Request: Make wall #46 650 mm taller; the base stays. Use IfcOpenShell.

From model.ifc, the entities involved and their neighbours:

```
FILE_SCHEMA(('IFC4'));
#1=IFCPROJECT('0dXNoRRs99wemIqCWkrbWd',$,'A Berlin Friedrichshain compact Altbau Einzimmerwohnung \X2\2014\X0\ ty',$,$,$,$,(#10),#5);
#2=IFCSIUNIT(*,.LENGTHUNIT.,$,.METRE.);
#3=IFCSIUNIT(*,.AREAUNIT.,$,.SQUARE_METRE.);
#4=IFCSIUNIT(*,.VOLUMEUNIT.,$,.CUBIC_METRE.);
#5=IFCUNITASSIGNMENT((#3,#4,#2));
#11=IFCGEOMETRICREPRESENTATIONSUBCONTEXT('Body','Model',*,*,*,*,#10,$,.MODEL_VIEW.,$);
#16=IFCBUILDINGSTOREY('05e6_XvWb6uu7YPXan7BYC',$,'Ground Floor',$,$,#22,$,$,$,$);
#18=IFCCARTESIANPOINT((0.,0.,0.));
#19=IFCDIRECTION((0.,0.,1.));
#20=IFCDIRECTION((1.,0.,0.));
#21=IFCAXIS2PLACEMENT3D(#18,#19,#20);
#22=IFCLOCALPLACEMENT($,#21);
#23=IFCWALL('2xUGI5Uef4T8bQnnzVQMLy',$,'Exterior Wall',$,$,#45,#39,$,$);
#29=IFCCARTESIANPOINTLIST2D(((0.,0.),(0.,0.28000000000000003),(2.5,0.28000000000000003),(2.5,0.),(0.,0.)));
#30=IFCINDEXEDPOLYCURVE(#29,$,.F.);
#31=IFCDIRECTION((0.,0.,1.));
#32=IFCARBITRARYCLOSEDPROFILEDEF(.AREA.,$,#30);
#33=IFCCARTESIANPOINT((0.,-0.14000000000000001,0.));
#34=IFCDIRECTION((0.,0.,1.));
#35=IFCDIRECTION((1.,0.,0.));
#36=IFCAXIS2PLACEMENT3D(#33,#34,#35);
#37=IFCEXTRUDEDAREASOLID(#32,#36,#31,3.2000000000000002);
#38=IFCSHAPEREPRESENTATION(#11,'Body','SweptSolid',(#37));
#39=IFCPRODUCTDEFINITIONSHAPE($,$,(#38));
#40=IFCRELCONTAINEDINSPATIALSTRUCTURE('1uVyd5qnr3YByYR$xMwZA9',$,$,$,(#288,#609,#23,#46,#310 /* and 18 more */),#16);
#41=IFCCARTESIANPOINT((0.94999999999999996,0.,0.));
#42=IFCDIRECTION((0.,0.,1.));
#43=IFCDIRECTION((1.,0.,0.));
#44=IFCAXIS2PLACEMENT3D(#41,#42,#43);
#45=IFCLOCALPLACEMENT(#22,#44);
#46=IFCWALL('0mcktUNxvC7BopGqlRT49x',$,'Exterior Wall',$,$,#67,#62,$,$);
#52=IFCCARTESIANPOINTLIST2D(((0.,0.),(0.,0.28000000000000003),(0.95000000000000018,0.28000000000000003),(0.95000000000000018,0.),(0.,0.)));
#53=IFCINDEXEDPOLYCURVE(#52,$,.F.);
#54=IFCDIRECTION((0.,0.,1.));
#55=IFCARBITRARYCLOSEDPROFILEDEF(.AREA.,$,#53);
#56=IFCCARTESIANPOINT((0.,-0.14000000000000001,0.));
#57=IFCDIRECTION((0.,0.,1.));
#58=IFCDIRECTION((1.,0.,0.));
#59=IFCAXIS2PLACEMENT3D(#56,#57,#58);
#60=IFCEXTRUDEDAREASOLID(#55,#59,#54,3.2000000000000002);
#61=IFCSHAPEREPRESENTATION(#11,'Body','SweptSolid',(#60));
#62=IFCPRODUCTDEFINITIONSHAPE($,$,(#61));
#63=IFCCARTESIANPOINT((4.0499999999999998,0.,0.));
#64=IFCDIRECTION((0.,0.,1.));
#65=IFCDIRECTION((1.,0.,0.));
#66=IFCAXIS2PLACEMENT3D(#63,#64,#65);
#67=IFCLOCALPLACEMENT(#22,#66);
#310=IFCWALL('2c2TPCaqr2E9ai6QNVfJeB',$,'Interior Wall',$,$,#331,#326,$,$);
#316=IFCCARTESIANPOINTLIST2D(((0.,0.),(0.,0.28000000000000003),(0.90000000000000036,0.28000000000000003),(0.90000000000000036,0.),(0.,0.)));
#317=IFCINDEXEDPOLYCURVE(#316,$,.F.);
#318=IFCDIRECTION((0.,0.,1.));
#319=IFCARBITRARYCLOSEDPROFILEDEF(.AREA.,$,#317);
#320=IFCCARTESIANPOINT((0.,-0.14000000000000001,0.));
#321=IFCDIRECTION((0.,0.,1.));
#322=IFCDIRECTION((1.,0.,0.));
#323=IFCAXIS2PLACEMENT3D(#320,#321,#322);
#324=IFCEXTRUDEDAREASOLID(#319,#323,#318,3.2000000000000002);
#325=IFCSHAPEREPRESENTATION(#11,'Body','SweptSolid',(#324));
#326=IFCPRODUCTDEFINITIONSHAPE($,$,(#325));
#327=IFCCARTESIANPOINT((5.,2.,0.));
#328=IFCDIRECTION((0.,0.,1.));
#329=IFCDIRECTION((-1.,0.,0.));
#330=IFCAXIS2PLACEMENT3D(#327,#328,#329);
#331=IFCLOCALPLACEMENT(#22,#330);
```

```python
import ifcopenshell
import ifcopenshell.geom
import ifcopenshell.util.representation
import ifcopenshell.util.shape
import ifcopenshell.util.unit

model = ifcopenshell.open("model.ifc")
unit_scale = ifcopenshell.util.unit.calculate_unit_scale(model)
settings = ifcopenshell.geom.settings()


def volume(element):
    """Net volume in cubic metres, openings subtracted."""
    shape = ifcopenshell.geom.create_shape(settings, element)
    return ifcopenshell.util.shape.get_volume(shape.geometry)


wall = model.by_guid("0mcktUNxvC7BopGqlRT49x")
before = volume(wall)

body = ifcopenshell.util.representation.get_representation(wall, "Model", "Body")
solid = body.Items[0]
old_height = solid.Depth
solid.Depth += 0.65 / unit_scale
after = volume(wall)

print(f"height {old_height:g} -> {solid.Depth:g}, volume {before:.3f} -> {after:.3f} m3")

model.write("model_updated.ifc")
```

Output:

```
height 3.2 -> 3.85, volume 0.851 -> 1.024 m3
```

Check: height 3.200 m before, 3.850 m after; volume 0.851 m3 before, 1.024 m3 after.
